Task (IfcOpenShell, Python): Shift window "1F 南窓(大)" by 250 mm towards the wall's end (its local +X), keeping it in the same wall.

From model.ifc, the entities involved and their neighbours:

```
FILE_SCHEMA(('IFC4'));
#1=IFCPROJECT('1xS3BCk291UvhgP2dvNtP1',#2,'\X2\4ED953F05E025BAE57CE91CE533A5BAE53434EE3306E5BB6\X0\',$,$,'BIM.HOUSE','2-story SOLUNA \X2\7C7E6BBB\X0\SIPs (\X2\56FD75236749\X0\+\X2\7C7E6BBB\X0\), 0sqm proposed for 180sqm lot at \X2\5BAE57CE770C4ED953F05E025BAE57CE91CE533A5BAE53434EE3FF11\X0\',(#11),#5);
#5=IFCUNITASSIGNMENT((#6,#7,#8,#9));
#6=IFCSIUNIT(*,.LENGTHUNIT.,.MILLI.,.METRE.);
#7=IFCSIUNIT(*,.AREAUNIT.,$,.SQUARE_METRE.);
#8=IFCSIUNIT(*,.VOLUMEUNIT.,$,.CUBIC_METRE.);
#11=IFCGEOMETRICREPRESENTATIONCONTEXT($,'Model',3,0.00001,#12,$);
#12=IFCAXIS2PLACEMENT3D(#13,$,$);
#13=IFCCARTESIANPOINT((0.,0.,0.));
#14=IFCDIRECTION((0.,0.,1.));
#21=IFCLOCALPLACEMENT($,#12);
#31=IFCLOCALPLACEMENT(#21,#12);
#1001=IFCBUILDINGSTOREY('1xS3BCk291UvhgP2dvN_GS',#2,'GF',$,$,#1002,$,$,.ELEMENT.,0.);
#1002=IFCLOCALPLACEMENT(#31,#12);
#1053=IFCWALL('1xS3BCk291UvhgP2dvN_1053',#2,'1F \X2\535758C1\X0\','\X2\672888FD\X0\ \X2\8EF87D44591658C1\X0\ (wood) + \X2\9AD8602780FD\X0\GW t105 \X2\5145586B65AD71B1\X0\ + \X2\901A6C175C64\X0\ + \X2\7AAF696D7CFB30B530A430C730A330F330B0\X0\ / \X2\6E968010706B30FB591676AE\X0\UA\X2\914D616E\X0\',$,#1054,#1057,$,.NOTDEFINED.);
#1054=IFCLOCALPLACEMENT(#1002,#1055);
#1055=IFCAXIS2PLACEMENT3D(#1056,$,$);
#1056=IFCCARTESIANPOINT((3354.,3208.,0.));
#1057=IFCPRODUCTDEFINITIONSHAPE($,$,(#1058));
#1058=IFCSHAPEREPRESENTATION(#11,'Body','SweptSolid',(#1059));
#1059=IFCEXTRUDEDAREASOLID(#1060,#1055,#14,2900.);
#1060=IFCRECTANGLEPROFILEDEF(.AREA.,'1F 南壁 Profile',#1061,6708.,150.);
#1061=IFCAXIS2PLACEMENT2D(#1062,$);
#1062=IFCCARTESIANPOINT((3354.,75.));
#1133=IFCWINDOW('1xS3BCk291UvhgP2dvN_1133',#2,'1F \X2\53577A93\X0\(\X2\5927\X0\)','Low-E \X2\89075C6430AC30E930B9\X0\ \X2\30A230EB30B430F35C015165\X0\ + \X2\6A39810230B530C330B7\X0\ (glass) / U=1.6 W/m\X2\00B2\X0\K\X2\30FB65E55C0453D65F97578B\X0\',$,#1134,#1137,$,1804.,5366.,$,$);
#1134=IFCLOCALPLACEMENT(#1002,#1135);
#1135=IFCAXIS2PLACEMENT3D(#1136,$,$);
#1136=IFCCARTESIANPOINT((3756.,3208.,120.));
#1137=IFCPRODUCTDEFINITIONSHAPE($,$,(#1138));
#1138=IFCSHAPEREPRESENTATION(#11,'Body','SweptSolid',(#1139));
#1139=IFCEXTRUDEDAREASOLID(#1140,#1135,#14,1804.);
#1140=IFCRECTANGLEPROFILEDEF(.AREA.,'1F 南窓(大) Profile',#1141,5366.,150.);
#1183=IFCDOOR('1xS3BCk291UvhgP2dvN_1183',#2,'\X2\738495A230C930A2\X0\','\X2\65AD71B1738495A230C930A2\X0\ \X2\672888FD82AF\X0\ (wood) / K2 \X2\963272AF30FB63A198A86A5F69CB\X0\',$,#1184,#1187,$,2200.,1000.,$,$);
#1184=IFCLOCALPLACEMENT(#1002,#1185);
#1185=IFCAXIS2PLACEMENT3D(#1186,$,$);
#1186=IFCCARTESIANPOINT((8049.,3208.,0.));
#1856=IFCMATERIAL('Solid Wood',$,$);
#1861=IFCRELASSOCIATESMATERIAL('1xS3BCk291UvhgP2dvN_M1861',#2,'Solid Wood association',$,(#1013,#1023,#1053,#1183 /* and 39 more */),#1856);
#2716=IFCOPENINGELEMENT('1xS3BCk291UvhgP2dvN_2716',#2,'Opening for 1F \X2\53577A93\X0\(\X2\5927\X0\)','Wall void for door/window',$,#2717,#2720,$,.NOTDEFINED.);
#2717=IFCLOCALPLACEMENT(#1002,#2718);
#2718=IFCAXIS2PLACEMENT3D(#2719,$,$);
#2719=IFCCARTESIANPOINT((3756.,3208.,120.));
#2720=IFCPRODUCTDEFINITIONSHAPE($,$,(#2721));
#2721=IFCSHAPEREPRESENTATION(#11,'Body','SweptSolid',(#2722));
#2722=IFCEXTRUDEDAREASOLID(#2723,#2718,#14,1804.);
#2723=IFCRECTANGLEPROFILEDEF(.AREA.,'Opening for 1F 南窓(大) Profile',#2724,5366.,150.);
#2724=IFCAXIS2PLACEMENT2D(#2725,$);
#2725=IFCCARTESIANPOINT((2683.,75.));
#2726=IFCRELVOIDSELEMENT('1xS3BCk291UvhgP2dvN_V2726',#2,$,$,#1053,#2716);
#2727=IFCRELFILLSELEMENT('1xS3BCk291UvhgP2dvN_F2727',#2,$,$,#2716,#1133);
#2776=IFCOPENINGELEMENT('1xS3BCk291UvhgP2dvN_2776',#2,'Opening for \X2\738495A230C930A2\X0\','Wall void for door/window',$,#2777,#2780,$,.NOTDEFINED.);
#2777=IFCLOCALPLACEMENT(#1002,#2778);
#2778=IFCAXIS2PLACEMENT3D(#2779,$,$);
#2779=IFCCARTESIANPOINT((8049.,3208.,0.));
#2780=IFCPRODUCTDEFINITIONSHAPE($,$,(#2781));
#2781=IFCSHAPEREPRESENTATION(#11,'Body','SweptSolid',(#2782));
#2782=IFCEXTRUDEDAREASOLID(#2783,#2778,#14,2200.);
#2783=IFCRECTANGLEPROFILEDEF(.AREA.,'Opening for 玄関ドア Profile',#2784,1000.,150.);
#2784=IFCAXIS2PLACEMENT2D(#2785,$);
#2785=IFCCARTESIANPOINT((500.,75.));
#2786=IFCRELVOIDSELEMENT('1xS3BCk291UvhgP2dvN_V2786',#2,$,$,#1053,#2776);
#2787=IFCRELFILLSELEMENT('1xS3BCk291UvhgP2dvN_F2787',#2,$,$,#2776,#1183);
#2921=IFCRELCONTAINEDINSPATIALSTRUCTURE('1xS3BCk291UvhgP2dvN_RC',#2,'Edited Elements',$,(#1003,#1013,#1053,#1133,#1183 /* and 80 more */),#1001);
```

```python
import ifcopenshell
import ifcopenshell.api.geometry
import ifcopenshell.util.placement
import ifcopenshell.util.unit

model = ifcopenshell.open("model.ifc")
unit_scale = ifcopenshell.util.unit.calculate_unit_scale(model)

window = model.by_guid("1xS3BCk291UvhgP2dvN_1133")
opening = window.FillsVoids[0].RelatingOpeningElement
wall = opening.VoidsElements[0].RelatingBuildingElement

wall_matrix = ifcopenshell.util.placement.get_local_placement(wall.ObjectPlacement)
shift = wall_matrix[:3, 0] * 0.25 / unit_scale
before = ifcopenshell.util.placement.get_local_placement(window.ObjectPlacement)[:3, 3].copy()

# The window is not placed relative to its opening, so move both.
for product in (opening, window):
    matrix = ifcopenshell.util.placement.get_local_placement(product.ObjectPlacement)
    matrix[:3, 3] += shift
    ifcopenshell.api.geometry.edit_object_placement(model, product=product, matrix=matrix, is_si=False)

after = ifcopenshell.util.placement.get_local_placement(window.ObjectPlacement)[:3, 3]
print("window moved by", (after - before).round(3) + 0.0)

model.write("model_updated.ifc")
```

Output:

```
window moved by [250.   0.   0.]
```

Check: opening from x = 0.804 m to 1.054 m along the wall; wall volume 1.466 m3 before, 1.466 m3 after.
